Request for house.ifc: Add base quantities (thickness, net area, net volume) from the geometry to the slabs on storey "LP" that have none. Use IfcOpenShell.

First a look at what the model holds.

```python
import ifcopenshell
import ifcopenshell.util.element
import ifcopenshell.util.unit

model = ifcopenshell.open("house.ifc")
print(model.schema)
for unit_type in ("LENGTHUNIT", "AREAUNIT", "VOLUMEUNIT"):
    print(unit_type, ifcopenshell.util.unit.calculate_unit_scale(model, unit_type))
storey = next(s for s in model.by_type("IfcBuildingStorey") if s.Name == "LP")
slabs = [e for e in ifcopenshell.util.element.get_decomposition(storey) if e.is_a("IfcSlab")]
for e in sorted(slabs, key=lambda e: e.id()):
    print(e.id(), e.is_a(), e.Name, list(ifcopenshell.util.element.get_psets(e, qtos_only=True)), sep=" | ")
```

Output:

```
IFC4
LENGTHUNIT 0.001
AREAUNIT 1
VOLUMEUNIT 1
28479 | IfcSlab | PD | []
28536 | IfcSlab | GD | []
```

```python
import ifcopenshell
import ifcopenshell.api.pset
import ifcopenshell.geom
import ifcopenshell.util.element
import ifcopenshell.util.shape
import ifcopenshell.util.unit

model = ifcopenshell.open("house.ifc")
unit_scale = ifcopenshell.util.unit.calculate_unit_scale(model)
area_scale = ifcopenshell.util.unit.calculate_unit_scale(model, "AREAUNIT")
volume_scale = ifcopenshell.util.unit.calculate_unit_scale(model, "VOLUMEUNIT")
settings = ifcopenshell.geom.settings()

storey = next(s for s in model.by_type("IfcBuildingStorey") if s.Name == "LP")
slabs = [e for e in ifcopenshell.util.element.get_decomposition(storey) if e.is_a("IfcSlab")]

for e in sorted(slabs, key=lambda e: e.id()):
    if ifcopenshell.util.element.get_psets(e, qtos_only=True, should_inherit=False):
        continue
    # Geometry comes back in metres, in the element's own axes.
    shape = ifcopenshell.geom.create_shape(settings, e)
    values = {
        "Width": ifcopenshell.util.shape.get_z(shape.geometry) / unit_scale,
        "NetArea": ifcopenshell.util.shape.get_footprint_area(shape.geometry) / area_scale,
        "NetVolume": ifcopenshell.util.shape.get_volume(shape.geometry) / volume_scale,
    }
    qto = ifcopenshell.api.pset.add_qto(model, product=e, name="Qto_SlabBaseQuantities")
    ifcopenshell.api.pset.edit_qto(model, qto=qto, properties=values)
    print(e.id(), {k: round(v, 3) for k, v in values.items()})

model.write("house_v2.ifc")
```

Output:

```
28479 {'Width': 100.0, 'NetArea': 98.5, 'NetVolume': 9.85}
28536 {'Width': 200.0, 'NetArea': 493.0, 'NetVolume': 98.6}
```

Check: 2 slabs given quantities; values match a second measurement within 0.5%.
